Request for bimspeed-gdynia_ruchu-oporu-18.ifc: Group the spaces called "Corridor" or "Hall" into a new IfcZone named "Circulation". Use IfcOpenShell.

First a look at what the model holds.

```python
import ifcopenshell

model = ifcopenshell.open("bimspeed-gdynia_ruchu-oporu-18.ifc")
print(model.schema)
seen = {}
for space in model.by_type("IfcSpace"):
    seen[space.LongName] = seen.get(space.LongName, 0) + 1
for name, count in sorted(seen.items(), key=str):
    print(count, "x", name)
print("zones:", [z.Name for z in model.by_type("IfcZone")][:20])
```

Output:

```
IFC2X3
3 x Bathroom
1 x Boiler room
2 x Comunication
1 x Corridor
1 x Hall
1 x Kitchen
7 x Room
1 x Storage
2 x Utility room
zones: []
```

```python
import ifcopenshell
import ifcopenshell.api.group
import ifcopenshell.api.root

model = ifcopenshell.open("bimspeed-gdynia_ruchu-oporu-18.ifc")

names = {"Corridor", "Hall"}
spaces = [s for s in model.by_type("IfcSpace") if s.LongName in names]

zone = ifcopenshell.api.root.create_entity(model, ifc_class="IfcZone", name="Circulation")
ifcopenshell.api.group.assign_group(model, products=spaces, group=zone)
print(len(spaces), "spaces in", zone.Name)

model.write("bimspeed-gdynia_ruchu-oporu-18_rev.ifc")
```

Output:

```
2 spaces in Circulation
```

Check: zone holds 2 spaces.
